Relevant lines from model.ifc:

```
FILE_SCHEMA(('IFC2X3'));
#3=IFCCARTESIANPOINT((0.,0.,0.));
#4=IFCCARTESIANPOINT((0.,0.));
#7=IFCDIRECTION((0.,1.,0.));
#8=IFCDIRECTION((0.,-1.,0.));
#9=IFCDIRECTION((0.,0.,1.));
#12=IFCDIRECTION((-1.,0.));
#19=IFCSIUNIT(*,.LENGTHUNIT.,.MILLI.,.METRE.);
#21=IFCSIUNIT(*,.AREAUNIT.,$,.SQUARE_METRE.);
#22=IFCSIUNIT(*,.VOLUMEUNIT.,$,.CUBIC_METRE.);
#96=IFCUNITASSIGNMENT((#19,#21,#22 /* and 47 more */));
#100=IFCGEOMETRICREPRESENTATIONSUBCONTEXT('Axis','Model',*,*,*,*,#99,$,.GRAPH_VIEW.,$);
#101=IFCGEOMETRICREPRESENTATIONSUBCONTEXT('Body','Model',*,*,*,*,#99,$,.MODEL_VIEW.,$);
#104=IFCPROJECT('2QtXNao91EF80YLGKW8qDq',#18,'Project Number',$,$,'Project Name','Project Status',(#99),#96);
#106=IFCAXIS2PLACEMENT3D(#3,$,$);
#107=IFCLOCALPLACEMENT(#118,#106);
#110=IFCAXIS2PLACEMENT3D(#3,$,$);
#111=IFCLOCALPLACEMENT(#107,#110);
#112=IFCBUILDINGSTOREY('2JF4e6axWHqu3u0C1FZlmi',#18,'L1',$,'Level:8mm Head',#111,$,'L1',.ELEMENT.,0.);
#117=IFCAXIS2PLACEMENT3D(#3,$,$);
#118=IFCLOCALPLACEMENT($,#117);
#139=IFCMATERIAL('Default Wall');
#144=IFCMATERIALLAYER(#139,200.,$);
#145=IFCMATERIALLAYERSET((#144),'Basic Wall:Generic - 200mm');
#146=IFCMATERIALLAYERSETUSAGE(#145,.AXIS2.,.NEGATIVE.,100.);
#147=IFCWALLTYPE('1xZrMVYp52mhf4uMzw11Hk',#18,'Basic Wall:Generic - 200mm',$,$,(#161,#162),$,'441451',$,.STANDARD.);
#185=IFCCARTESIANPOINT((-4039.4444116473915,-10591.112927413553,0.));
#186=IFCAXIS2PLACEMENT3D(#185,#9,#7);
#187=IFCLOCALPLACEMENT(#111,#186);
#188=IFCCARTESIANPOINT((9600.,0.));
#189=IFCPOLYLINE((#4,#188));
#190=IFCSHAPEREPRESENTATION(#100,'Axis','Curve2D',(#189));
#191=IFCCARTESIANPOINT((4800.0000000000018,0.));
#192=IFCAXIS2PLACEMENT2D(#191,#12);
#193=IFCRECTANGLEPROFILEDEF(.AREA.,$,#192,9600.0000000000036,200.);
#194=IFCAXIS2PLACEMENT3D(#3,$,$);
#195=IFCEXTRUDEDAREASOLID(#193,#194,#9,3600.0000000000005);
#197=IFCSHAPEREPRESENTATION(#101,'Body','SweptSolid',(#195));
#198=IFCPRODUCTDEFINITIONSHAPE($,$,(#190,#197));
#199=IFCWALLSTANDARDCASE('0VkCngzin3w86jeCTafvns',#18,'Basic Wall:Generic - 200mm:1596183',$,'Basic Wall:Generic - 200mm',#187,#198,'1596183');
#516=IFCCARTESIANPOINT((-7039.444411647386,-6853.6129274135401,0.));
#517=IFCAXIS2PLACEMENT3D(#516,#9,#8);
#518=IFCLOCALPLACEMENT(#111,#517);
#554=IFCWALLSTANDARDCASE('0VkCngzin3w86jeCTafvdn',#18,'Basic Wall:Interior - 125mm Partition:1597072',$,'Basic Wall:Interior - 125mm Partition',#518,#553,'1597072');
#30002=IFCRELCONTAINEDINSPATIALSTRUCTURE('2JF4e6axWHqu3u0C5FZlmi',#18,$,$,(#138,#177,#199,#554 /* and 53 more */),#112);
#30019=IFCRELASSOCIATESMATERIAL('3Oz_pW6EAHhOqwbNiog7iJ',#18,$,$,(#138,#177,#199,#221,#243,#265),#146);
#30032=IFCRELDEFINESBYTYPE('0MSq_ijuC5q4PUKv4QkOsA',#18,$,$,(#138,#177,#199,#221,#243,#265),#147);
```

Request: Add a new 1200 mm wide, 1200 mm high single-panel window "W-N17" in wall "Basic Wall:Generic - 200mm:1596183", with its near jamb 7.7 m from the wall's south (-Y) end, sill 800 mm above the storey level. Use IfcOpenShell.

```python
import numpy as np
import ifcopenshell
import ifcopenshell.api.feature
import ifcopenshell.api.geometry
import ifcopenshell.api.root
import ifcopenshell.api.spatial
import ifcopenshell.api.type
import ifcopenshell.geom
import ifcopenshell.util.element
import ifcopenshell.util.placement
import ifcopenshell.util.representation
import ifcopenshell.util.shape
import ifcopenshell.util.unit

model = ifcopenshell.open("model.ifc")
unit_scale = ifcopenshell.util.unit.calculate_unit_scale(model)
settings = ifcopenshell.geom.settings()


def volume(element):
    """Net volume in cubic metres, openings subtracted."""
    shape = ifcopenshell.geom.create_shape(settings, element)
    return ifcopenshell.util.shape.get_volume(shape.geometry)


wall = model.by_guid("0VkCngzin3w86jeCTafvns")
storey = ifcopenshell.util.element.get_container(wall, ifc_class="IfcBuildingStorey")
context = ifcopenshell.util.representation.get_context(model, "Model", "Body", "MODEL_VIEW")
before = volume(wall)

width, height, from_end, sill = 1.2, 1.2, 7.7, 0.8  # metres

# The wall runs along its own X axis, and the end named is its -X end.
wall_shape = ifcopenshell.geom.create_shape(settings, wall)
x, y, z = ifcopenshell.util.shape.get_vertices(wall_shape.geometry).T
start = x.min() + from_end
face, thickness = float(y.min()), float(y.max() - y.min())
wall_matrix = ifcopenshell.util.placement.get_local_placement(wall.ObjectPlacement)
level = ifcopenshell.util.placement.get_local_placement(storey.ObjectPlacement)[2, 3]


def in_wall(x, y):
    """Placement at x, y metres in the wall's axes, at sill height."""
    matrix = wall_matrix.copy()
    matrix[:, 3] = wall_matrix @ np.array([x / unit_scale, y / unit_scale, 0.0, 1.0])
    matrix[2, 3] = level + sill / unit_scale
    return matrix


# Opening: a box that overshoots both wall faces by 50 mm.
opening = ifcopenshell.api.root.create_entity(model, ifc_class="IfcOpeningElement")
box = ifcopenshell.api.geometry.add_wall_representation(
    model, context=context, length=width, height=height, thickness=thickness + 0.1
)
ifcopenshell.api.geometry.assign_representation(model, product=opening, representation=box)
ifcopenshell.api.geometry.edit_object_placement(model, product=opening, matrix=in_wall(start, face - 0.05), is_si=False)
ifcopenshell.api.feature.add_feature(model, feature=opening, element=wall)

window = ifcopenshell.api.root.create_entity(model, ifc_class="IfcWindow", name="W-N17")
window.OverallWidth, window.OverallHeight = width / unit_scale, height / unit_scale
body = ifcopenshell.api.geometry.add_window_representation(
    model,
    context=context,
    overall_width=window.OverallWidth,
    overall_height=window.OverallHeight,
    partition_type="SINGLE_PANEL",
)
ifcopenshell.api.geometry.assign_representation(model, product=window, representation=body)
ifcopenshell.api.spatial.assign_container(model, products=[window], relating_structure=storey)
fills = ifcopenshell.api.feature.add_filling(model, opening=opening, element=window)
fills.OwnerHistory = window.OwnerHistory  # required in IFC2X3

# IFC2X3 keeps the operation on the window style.
style = ifcopenshell.api.root.create_entity(model, ifc_class="IfcWindowStyle", name="W-N17")
style.OperationType, style.ConstructionType = "SINGLE_PANEL", "NOTDEFINED"
style.ParameterTakesPrecedence = style.Sizeable = False
ifcopenshell.api.type.assign_type(model, related_objects=[window], relating_type=style)

# Centre the window in the wall's thickness.
ifcopenshell.api.geometry.edit_object_placement(model, product=window, matrix=in_wall(start, face), is_si=False)
window_shape = ifcopenshell.geom.create_shape(settings, window)
depth = ifcopenshell.util.shape.get_vertices(window_shape.geometry)[:, 1]
offset = face + thickness / 2 - (depth.min() + depth.max()) / 2
ifcopenshell.api.geometry.edit_object_placement(model, product=window, matrix=in_wall(start, offset), is_si=False)

after = volume(wall)

print(f"wall volume {before:.3f} -> {after:.3f} m3")

model.write("model_updated.ifc")
```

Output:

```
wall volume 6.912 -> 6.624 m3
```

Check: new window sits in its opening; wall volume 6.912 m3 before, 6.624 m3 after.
